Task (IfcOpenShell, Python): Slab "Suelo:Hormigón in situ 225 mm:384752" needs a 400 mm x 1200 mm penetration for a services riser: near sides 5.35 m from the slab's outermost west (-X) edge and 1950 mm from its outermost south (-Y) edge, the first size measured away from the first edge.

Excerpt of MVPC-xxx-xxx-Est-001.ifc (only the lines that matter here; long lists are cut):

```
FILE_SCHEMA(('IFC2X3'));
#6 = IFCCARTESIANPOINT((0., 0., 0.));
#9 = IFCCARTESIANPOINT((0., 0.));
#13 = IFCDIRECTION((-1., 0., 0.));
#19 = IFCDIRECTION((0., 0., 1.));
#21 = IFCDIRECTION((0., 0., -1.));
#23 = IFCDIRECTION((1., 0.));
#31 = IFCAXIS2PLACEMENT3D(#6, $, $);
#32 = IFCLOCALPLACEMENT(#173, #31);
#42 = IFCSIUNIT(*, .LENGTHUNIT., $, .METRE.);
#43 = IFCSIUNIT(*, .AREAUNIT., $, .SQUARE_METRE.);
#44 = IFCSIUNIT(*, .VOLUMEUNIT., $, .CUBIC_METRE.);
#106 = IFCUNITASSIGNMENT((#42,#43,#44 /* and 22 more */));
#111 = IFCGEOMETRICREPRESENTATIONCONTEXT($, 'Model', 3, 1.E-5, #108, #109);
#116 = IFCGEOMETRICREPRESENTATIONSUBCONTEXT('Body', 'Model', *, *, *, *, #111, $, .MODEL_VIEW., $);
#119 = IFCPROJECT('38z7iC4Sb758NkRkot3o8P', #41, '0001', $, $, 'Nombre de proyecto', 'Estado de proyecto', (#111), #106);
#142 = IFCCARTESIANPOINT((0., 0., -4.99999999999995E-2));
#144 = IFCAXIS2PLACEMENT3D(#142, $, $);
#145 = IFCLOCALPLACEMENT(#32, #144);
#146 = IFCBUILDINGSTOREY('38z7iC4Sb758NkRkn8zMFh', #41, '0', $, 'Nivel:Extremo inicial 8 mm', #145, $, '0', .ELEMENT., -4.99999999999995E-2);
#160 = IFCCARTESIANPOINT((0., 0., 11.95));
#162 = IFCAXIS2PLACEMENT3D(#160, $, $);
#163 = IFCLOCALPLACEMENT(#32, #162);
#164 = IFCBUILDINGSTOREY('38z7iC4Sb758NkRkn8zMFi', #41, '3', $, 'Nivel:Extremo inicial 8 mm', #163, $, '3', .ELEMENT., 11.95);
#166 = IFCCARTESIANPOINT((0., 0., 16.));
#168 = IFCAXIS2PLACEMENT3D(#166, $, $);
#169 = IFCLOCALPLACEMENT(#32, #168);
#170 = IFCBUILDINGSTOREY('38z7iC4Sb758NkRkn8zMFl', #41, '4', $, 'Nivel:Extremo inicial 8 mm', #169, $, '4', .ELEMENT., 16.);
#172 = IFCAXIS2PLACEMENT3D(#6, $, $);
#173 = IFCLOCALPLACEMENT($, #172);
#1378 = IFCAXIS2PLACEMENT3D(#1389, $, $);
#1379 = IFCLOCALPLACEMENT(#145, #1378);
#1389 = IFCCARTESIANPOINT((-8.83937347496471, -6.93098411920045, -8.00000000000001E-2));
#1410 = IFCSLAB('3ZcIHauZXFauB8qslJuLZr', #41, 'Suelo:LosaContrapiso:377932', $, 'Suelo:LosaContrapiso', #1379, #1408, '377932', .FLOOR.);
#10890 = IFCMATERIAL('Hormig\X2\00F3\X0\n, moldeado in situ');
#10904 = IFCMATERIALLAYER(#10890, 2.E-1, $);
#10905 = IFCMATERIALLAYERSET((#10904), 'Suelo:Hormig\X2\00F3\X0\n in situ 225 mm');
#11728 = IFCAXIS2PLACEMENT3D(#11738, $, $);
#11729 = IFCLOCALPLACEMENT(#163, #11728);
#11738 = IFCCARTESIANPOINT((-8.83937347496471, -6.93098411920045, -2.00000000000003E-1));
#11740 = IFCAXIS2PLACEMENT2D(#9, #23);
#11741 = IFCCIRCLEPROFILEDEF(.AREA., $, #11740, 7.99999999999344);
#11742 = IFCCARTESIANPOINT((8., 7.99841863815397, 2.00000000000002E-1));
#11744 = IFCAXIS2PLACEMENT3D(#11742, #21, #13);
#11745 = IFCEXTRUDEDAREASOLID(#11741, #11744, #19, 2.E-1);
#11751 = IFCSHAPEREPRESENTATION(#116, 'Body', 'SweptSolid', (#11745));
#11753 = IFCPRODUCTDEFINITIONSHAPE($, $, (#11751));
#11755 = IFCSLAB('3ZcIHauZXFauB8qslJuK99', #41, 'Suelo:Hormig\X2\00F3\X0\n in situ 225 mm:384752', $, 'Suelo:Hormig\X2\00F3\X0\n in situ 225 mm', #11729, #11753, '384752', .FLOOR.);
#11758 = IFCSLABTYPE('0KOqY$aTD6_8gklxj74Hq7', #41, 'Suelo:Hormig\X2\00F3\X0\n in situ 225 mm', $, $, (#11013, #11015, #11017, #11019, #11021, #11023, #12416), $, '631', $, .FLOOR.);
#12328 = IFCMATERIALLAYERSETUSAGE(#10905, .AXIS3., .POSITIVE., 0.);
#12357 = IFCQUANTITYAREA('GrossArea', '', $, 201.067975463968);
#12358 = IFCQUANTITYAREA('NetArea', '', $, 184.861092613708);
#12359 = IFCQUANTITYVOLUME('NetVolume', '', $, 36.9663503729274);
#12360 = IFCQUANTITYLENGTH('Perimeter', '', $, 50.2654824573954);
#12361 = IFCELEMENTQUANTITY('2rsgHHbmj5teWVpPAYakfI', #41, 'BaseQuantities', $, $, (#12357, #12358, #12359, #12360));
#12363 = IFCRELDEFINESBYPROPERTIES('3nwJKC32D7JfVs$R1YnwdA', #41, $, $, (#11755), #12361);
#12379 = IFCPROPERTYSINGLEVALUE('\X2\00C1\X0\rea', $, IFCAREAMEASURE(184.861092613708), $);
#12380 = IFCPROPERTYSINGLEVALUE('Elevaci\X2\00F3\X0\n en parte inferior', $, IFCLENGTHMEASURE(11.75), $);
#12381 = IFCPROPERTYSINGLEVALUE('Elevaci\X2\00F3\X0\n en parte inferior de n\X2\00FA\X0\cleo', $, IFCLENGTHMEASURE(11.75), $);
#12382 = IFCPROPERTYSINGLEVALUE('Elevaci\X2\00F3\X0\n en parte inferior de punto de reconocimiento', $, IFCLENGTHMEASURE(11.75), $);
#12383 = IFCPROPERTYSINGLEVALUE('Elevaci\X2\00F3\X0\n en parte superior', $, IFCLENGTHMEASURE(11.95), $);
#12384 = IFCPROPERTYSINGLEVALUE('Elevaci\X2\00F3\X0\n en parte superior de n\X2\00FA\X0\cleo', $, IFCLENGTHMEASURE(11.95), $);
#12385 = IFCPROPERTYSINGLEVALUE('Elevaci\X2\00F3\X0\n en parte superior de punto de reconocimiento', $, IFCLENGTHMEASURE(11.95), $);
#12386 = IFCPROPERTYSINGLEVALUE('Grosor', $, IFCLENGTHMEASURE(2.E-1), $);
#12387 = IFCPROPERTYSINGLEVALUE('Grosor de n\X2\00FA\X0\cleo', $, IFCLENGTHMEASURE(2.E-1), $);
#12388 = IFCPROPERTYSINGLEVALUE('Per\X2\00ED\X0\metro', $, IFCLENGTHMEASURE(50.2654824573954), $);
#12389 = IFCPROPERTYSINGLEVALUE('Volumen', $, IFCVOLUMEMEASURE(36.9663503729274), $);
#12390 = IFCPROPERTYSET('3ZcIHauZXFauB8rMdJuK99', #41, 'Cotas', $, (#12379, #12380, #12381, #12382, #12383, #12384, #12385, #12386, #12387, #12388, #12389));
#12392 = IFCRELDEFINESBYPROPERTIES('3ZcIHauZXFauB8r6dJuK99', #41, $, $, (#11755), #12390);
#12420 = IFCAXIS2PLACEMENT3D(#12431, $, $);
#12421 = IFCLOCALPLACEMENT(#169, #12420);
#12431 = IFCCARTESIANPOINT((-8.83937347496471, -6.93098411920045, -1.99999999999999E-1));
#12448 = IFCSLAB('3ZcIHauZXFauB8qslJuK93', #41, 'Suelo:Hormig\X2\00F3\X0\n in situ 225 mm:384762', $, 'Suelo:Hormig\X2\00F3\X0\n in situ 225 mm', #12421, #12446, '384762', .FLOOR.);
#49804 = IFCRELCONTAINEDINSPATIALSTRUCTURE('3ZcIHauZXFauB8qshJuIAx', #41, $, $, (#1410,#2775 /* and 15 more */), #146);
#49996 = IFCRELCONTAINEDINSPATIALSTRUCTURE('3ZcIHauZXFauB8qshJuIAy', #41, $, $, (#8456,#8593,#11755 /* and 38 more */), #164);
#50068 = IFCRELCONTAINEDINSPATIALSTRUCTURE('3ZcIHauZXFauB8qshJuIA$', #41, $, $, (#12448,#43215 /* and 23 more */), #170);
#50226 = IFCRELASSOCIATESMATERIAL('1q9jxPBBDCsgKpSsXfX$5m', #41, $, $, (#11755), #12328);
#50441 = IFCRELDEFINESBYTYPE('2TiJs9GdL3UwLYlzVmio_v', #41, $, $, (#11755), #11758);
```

```python
import numpy as np
import ifcopenshell
import ifcopenshell.api.feature
import ifcopenshell.api.geometry
import ifcopenshell.api.pset
import ifcopenshell.api.root
import ifcopenshell.geom
import ifcopenshell.util.element
import ifcopenshell.util.placement
import ifcopenshell.util.representation
import ifcopenshell.util.shape
import ifcopenshell.util.unit

model = ifcopenshell.open("MVPC-xxx-xxx-Est-001.ifc")
unit_scale = ifcopenshell.util.unit.calculate_unit_scale(model)
area_scale = ifcopenshell.util.unit.calculate_unit_scale(model, "AREAUNIT")
volume_scale = ifcopenshell.util.unit.calculate_unit_scale(model, "VOLUMEUNIT")
settings = ifcopenshell.geom.settings()


def volume(element):
    """Net volume in cubic metres, openings subtracted."""
    shape = ifcopenshell.geom.create_shape(settings, element)
    return ifcopenshell.util.shape.get_volume(shape.geometry)


slab = model.by_id(11755)
before = volume(slab)

# Extent in the slab's own axes, in metres. The edges named are its -X and -Y sides.
slab_shape = ifcopenshell.geom.create_shape(settings, slab)
vertices = ifcopenshell.util.shape.get_vertices(slab_shape.geometry)
x_min, y_min, bottom = vertices.min(axis=0)
top = vertices[:, 2].max()

opening = ifcopenshell.api.root.create_entity(model, ifc_class="IfcOpeningElement", name="Services riser opening")
context = ifcopenshell.util.representation.get_context(model, "Model", "Body", "MODEL_VIEW")
width, depth = 0.4, 1.2
outline = [(0.0, 0.0), (width, 0.0), (width, depth), (0.0, depth), (0.0, 0.0)]
# Overshoot both faces by 50 mm so the cut is clean.
shape = ifcopenshell.api.geometry.add_slab_representation(
    model, context=context, depth=top - bottom + 0.1, polyline=outline
)
ifcopenshell.api.geometry.assign_representation(model, product=opening, representation=shape)

matrix = ifcopenshell.util.placement.get_local_placement(slab.ObjectPlacement)
matrix[:, 3] = matrix @ np.append(np.array([x_min + 5.35, y_min + 1.95, bottom - 0.05]) / unit_scale, 1.0)
ifcopenshell.api.geometry.edit_object_placement(model, product=opening, matrix=matrix, is_si=False)
ifcopenshell.api.feature.add_feature(model, feature=opening, element=slab)

after = volume(slab)

# Update the slab's stored quantities.
qto = model.by_id(ifcopenshell.util.element.get_pset(slab, "BaseQuantities", should_inherit=False)["id"])
ifcopenshell.api.pset.edit_qto(model, qto=qto, properties={
    "NetArea": after / (top - bottom) / area_scale,
    "NetVolume": after / volume_scale,
})
pset = model.by_id(ifcopenshell.util.element.get_pset(slab, "Cotas", should_inherit=False)["id"])
ifcopenshell.api.pset.edit_pset(model, pset=pset, properties={
    "Área": model.create_entity("IfcAreaMeasure", after / (top - bottom) / area_scale),
    "Volumen": model.create_entity("IfcVolumeMeasure", after / volume_scale),
})

print(f"slab volume {before:.3f} -> {after:.3f} m3")

model.write("MVPC-xxx-xxx-Est-001_rev.ifc")
```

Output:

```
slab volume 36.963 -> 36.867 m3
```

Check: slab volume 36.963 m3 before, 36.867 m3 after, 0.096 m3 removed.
